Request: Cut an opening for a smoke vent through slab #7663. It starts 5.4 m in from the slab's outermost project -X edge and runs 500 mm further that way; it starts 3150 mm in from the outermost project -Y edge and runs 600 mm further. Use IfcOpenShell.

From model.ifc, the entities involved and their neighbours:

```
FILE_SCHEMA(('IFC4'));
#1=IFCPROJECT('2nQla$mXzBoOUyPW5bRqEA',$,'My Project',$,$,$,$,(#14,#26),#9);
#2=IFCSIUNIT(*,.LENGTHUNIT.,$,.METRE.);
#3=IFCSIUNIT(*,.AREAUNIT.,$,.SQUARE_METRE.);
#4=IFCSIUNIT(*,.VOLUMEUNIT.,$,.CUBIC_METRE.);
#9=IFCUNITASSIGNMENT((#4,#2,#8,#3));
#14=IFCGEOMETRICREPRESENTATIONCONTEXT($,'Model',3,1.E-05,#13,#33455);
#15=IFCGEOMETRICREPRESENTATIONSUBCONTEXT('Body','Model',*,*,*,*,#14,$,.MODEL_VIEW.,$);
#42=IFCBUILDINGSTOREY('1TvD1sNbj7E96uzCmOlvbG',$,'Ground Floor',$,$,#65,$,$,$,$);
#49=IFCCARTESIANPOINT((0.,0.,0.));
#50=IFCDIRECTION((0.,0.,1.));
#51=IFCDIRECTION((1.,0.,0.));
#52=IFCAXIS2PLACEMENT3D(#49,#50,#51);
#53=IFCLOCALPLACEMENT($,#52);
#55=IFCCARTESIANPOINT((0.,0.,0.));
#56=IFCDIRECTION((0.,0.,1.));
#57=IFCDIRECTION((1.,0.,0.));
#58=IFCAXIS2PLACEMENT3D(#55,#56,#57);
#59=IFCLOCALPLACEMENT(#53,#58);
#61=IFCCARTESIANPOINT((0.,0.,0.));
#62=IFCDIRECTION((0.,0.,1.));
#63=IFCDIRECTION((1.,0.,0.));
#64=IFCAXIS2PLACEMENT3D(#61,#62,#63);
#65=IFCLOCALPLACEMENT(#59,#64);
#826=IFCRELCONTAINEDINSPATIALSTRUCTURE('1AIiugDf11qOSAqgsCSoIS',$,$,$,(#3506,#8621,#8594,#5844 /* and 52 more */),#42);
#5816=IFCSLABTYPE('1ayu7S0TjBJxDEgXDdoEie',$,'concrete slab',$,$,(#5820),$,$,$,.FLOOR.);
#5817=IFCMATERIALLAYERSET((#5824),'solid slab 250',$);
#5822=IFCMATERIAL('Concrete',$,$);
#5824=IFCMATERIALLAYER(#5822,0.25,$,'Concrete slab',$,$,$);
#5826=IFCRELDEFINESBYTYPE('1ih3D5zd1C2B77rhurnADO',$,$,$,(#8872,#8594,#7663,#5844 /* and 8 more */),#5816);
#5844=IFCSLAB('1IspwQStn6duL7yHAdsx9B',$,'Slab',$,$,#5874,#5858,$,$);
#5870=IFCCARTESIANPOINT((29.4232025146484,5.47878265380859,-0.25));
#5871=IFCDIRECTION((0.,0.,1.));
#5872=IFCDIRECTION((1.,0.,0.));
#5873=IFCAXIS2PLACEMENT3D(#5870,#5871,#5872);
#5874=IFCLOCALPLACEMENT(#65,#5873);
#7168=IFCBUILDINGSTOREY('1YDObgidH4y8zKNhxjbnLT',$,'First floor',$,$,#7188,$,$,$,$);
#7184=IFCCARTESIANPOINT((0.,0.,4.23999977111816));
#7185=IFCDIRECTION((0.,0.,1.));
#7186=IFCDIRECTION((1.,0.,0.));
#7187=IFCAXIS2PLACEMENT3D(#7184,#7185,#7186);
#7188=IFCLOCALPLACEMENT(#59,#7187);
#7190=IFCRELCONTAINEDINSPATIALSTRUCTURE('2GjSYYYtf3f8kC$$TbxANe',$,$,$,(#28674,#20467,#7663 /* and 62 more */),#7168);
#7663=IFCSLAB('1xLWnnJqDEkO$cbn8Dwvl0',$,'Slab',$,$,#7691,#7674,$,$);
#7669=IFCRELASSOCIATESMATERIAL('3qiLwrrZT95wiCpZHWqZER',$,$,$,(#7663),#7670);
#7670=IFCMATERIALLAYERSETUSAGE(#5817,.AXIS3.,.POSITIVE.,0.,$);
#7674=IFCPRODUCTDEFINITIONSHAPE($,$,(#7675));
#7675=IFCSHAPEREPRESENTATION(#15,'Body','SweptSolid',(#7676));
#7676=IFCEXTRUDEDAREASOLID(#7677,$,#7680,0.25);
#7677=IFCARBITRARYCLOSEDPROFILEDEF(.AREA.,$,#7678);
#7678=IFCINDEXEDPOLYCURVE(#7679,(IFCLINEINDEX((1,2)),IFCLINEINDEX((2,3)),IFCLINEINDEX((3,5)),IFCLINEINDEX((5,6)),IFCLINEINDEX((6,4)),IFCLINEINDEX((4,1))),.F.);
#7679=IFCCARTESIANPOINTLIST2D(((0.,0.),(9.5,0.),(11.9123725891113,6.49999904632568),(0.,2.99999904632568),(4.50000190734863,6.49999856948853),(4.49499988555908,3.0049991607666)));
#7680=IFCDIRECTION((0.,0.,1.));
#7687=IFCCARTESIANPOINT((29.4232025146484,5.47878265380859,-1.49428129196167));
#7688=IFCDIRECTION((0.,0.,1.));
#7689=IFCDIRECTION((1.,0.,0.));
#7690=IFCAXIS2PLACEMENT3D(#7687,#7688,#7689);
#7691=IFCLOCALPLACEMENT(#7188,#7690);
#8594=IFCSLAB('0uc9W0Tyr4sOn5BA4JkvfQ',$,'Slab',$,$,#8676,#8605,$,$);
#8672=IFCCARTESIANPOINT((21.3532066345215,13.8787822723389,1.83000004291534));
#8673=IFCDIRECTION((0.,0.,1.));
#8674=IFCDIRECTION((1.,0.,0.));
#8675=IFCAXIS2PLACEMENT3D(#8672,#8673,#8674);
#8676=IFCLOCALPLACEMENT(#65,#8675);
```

```python
import numpy as np
import ifcopenshell
import ifcopenshell.api.feature
import ifcopenshell.api.geometry
import ifcopenshell.api.root
import ifcopenshell.geom
import ifcopenshell.util.placement
import ifcopenshell.util.representation
import ifcopenshell.util.shape
import ifcopenshell.util.unit

model = ifcopenshell.open("model.ifc")
unit_scale = ifcopenshell.util.unit.calculate_unit_scale(model)
settings = ifcopenshell.geom.settings()


def volume(element):
    """Net volume in cubic metres, openings subtracted."""
    shape = ifcopenshell.geom.create_shape(settings, element)
    return ifcopenshell.util.shape.get_volume(shape.geometry)


slab = model.by_guid("1xLWnnJqDEkO$cbn8Dwvl0")
before = volume(slab)

# Extent in the slab's own axes, in metres. The edges named are its -X and -Y sides.
slab_shape = ifcopenshell.geom.create_shape(settings, slab)
vertices = ifcopenshell.util.shape.get_vertices(slab_shape.geometry)
x_min, y_min, bottom = vertices.min(axis=0)
top = vertices[:, 2].max()

opening = ifcopenshell.api.root.create_entity(model, ifc_class="IfcOpeningElement", name="Smoke vent opening", predefined_type="OPENING")
context = ifcopenshell.util.representation.get_context(model, "Model", "Body", "MODEL_VIEW")
width, depth = 0.5, 0.6
outline = [(0.0, 0.0), (width, 0.0), (width, depth), (0.0, depth), (0.0, 0.0)]
# Overshoot both faces by 50 mm so the cut is clean.
shape = ifcopenshell.api.geometry.add_slab_representation(
    model, context=context, depth=top - bottom + 0.1, polyline=outline
)
ifcopenshell.api.geometry.assign_representation(model, product=opening, representation=shape)

matrix = ifcopenshell.util.placement.get_local_placement(slab.ObjectPlacement)
matrix[:, 3] = matrix @ np.append(np.array([x_min + 5.4, y_min + 3.15, bottom - 0.05]) / unit_scale, 1.0)
ifcopenshell.api.geometry.edit_object_placement(model, product=opening, matrix=matrix, is_si=False)
ifcopenshell.api.feature.add_feature(model, feature=opening, element=slab)

after = volume(slab)

print(f"slab volume {before:.3f} -> {after:.3f} m3")

model.write("model-out.ifc")
```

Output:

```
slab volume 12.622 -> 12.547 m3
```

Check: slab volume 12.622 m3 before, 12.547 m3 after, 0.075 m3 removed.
